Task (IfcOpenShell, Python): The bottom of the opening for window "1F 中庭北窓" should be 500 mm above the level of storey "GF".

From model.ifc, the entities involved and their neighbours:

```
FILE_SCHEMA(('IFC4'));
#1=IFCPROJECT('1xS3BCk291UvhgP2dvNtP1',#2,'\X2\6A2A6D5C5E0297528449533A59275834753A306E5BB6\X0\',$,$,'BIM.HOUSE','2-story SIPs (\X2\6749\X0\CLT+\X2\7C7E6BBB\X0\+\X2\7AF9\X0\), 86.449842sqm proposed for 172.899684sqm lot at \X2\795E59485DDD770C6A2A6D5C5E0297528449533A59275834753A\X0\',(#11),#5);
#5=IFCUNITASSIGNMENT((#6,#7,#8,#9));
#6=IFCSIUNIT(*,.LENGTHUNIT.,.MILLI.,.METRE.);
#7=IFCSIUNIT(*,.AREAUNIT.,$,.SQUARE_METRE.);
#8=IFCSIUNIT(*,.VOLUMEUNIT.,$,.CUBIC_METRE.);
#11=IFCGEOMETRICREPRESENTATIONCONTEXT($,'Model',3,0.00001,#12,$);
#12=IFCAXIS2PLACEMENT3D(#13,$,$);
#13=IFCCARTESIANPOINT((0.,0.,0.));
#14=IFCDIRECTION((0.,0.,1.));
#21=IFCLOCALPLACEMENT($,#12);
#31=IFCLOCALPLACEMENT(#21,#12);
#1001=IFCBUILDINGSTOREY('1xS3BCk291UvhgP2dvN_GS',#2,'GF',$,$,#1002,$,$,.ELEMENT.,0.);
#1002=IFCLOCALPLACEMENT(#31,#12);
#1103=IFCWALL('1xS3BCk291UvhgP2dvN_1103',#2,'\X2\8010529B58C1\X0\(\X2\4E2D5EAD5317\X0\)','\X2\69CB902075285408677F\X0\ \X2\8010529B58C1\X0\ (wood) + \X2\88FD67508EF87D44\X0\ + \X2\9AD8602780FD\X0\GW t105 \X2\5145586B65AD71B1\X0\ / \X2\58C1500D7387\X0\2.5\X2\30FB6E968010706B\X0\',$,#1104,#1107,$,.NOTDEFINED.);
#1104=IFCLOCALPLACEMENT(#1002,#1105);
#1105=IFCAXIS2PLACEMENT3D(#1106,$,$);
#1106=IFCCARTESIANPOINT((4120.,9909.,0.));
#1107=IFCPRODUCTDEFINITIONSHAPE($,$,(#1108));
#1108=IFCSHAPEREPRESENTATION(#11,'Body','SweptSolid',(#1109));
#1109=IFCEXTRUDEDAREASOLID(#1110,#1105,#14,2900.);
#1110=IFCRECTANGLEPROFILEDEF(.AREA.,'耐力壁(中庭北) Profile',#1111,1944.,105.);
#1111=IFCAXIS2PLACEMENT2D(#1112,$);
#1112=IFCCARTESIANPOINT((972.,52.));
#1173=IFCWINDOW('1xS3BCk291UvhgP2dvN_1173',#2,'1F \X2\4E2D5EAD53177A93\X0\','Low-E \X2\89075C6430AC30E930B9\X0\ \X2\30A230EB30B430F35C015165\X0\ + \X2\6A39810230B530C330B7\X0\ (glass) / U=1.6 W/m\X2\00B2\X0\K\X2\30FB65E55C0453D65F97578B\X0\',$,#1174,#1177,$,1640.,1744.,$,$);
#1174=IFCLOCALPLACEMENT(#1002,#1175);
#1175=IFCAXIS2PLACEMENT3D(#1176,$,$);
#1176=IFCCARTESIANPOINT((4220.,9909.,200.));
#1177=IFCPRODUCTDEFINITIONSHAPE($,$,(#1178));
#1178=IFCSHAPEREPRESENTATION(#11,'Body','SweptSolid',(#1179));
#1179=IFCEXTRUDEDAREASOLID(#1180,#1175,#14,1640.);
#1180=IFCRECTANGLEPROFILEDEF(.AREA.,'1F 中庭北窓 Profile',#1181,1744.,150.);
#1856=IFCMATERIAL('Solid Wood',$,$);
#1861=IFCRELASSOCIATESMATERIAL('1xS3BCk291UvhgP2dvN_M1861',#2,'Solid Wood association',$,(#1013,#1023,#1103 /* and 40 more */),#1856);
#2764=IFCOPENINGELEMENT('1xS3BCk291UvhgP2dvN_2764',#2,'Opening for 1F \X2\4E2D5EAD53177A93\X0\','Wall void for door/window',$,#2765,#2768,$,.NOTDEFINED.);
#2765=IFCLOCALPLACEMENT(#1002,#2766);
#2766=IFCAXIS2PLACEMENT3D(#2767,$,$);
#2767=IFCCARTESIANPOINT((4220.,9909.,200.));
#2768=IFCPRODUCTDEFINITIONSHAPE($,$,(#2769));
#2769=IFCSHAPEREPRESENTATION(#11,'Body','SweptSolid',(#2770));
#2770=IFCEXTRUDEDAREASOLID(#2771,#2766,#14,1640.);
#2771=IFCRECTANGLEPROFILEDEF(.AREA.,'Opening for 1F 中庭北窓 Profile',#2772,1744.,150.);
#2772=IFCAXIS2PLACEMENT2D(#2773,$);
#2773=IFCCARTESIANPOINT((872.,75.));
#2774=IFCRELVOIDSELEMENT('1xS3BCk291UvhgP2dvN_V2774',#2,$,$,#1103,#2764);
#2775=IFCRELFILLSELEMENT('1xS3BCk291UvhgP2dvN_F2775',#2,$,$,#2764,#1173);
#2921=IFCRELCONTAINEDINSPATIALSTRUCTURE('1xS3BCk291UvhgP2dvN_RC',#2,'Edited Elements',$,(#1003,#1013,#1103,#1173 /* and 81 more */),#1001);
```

```python
import numpy as np
import ifcopenshell
import ifcopenshell.api.geometry
import ifcopenshell.geom
import ifcopenshell.util.element
import ifcopenshell.util.placement
import ifcopenshell.util.shape
import ifcopenshell.util.unit

model = ifcopenshell.open("model.ifc")
unit_scale = ifcopenshell.util.unit.calculate_unit_scale(model)

window = model.by_guid("1xS3BCk291UvhgP2dvN_1173")
opening = window.FillsVoids[0].RelatingOpeningElement
storey = ifcopenshell.util.element.get_container(window, ifc_class="IfcBuildingStorey")
level = ifcopenshell.util.placement.get_local_placement(storey.ObjectPlacement)[2, 3]

# The opening's origin need not be at the sill, so measure its lowest point.
shape = ifcopenshell.geom.create_shape(ifcopenshell.geom.settings(), opening)
bottom = ifcopenshell.util.shape.get_shape_bottom_elevation(shape, shape.geometry) / unit_scale
dz = level + 0.5 / unit_scale - bottom

shift = np.array([0.0, 0.0, dz])
# The window is not placed relative to its opening, so move both.
for product in (opening, window):
    matrix = ifcopenshell.util.placement.get_local_placement(product.ObjectPlacement)
    matrix[:3, 3] += shift
    ifcopenshell.api.geometry.edit_object_placement(model, product=product, matrix=matrix, is_si=False)

print(f"moved by {dz * unit_scale:+.3f} m")

model.write("model_rev.ifc")
```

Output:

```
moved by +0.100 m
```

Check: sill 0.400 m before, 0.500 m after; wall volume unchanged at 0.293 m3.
